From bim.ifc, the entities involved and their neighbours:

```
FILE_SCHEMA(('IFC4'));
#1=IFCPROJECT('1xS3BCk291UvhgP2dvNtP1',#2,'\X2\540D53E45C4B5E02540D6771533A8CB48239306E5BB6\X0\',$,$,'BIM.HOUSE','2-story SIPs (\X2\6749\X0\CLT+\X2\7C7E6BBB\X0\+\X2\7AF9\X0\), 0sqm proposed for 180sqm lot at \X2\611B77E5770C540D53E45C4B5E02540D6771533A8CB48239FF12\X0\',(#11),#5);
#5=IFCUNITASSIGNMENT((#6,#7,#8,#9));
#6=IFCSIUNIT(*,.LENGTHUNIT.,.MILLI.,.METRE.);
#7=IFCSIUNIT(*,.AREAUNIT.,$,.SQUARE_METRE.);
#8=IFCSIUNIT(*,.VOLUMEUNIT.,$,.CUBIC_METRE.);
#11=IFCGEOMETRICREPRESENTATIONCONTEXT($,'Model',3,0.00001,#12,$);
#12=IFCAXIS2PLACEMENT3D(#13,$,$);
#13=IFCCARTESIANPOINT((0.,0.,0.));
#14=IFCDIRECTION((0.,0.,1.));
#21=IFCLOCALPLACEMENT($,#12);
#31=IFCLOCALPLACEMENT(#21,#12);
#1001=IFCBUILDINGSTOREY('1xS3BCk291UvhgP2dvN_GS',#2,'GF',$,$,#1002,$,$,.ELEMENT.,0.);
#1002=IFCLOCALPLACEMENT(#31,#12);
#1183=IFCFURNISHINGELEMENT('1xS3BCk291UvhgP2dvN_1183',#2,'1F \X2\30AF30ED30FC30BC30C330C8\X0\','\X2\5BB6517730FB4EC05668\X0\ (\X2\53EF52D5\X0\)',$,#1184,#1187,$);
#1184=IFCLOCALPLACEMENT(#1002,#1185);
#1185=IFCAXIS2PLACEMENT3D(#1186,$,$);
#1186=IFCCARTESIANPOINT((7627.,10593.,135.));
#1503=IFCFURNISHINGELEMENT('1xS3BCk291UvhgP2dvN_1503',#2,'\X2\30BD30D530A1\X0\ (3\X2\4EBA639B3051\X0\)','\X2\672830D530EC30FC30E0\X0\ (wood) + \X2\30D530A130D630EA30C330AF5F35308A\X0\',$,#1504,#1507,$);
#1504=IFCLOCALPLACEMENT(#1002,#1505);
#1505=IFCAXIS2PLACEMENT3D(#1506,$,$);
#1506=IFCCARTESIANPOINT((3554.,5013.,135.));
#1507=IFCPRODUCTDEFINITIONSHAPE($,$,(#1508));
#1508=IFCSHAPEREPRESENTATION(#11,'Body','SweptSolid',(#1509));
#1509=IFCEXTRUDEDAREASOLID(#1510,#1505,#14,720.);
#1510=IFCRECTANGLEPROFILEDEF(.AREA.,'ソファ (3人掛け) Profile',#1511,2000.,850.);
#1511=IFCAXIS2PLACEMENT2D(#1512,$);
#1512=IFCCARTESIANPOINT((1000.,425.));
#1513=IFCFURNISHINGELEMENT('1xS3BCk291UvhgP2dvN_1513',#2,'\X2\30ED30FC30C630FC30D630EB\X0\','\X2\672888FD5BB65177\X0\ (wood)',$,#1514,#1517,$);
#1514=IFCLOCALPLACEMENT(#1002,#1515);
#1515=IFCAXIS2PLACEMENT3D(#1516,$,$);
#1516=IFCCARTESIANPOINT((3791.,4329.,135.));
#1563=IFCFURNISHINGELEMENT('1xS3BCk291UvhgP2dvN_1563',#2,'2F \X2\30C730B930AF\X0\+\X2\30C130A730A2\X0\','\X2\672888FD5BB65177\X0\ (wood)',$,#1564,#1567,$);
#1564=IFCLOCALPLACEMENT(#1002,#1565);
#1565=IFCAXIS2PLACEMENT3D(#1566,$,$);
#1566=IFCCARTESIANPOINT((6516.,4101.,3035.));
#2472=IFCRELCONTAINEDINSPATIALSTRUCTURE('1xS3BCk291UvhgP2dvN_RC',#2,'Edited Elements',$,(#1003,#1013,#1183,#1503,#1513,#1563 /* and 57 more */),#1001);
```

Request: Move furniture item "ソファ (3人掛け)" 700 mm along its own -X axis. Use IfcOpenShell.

```python
import ifcopenshell
import ifcopenshell.api.geometry
import ifcopenshell.util.placement

model = ifcopenshell.open("bim.ifc")

item = model.by_guid("1xS3BCk291UvhgP2dvN_1503")
matrix = ifcopenshell.util.placement.get_local_placement(item.ObjectPlacement)
matrix[:3, 3] -= matrix[:3, 0] * 700.0
ifcopenshell.api.geometry.edit_object_placement(model, product=item, matrix=matrix, is_si=False)

print(ifcopenshell.util.placement.get_local_placement(item.ObjectPlacement).round(3) + 0.0)

model.write("bim_rev.ifc")
```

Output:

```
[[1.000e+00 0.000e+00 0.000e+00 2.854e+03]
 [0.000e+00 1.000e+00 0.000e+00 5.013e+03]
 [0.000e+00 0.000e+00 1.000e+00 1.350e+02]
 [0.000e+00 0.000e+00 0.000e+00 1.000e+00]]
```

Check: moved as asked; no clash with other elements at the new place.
